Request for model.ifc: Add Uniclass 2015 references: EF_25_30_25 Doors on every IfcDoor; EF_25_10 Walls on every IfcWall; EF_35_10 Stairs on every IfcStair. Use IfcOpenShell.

First a look at what the model holds.

```python
import ifcopenshell

model = ifcopenshell.open("model.ifc")
print(model.schema)
print("classifications:", [c.Name for c in model.by_type("IfcClassification")])
for ifc_class in ("IfcDoor", "IfcRoof", "IfcStair", "IfcWall", "IfcWindow"):
    print(ifc_class, len(model.by_type(ifc_class)))
```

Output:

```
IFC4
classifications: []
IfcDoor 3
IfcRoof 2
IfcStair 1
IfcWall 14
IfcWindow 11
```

```python
import ifcopenshell
import ifcopenshell.api.classification

model = ifcopenshell.open("model.ifc")

system = ifcopenshell.api.classification.add_classification(model, classification="Uniclass 2015")

codes = {
    "IfcDoor": ("EF_25_30_25", "Doors"),
    "IfcWall": ("EF_25_10", "Walls"),
    "IfcStair": ("EF_35_10", "Stairs"),
}
for ifc_class, (code, name) in codes.items():
    products = model.by_type(ifc_class)
    ifcopenshell.api.classification.add_reference(
        model, products=products, classification=system, identification=code, name=name
    )
    print(code, len(products))

model.write("model_edited.ifc")
```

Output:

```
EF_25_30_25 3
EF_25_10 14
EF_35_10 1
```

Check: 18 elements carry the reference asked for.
